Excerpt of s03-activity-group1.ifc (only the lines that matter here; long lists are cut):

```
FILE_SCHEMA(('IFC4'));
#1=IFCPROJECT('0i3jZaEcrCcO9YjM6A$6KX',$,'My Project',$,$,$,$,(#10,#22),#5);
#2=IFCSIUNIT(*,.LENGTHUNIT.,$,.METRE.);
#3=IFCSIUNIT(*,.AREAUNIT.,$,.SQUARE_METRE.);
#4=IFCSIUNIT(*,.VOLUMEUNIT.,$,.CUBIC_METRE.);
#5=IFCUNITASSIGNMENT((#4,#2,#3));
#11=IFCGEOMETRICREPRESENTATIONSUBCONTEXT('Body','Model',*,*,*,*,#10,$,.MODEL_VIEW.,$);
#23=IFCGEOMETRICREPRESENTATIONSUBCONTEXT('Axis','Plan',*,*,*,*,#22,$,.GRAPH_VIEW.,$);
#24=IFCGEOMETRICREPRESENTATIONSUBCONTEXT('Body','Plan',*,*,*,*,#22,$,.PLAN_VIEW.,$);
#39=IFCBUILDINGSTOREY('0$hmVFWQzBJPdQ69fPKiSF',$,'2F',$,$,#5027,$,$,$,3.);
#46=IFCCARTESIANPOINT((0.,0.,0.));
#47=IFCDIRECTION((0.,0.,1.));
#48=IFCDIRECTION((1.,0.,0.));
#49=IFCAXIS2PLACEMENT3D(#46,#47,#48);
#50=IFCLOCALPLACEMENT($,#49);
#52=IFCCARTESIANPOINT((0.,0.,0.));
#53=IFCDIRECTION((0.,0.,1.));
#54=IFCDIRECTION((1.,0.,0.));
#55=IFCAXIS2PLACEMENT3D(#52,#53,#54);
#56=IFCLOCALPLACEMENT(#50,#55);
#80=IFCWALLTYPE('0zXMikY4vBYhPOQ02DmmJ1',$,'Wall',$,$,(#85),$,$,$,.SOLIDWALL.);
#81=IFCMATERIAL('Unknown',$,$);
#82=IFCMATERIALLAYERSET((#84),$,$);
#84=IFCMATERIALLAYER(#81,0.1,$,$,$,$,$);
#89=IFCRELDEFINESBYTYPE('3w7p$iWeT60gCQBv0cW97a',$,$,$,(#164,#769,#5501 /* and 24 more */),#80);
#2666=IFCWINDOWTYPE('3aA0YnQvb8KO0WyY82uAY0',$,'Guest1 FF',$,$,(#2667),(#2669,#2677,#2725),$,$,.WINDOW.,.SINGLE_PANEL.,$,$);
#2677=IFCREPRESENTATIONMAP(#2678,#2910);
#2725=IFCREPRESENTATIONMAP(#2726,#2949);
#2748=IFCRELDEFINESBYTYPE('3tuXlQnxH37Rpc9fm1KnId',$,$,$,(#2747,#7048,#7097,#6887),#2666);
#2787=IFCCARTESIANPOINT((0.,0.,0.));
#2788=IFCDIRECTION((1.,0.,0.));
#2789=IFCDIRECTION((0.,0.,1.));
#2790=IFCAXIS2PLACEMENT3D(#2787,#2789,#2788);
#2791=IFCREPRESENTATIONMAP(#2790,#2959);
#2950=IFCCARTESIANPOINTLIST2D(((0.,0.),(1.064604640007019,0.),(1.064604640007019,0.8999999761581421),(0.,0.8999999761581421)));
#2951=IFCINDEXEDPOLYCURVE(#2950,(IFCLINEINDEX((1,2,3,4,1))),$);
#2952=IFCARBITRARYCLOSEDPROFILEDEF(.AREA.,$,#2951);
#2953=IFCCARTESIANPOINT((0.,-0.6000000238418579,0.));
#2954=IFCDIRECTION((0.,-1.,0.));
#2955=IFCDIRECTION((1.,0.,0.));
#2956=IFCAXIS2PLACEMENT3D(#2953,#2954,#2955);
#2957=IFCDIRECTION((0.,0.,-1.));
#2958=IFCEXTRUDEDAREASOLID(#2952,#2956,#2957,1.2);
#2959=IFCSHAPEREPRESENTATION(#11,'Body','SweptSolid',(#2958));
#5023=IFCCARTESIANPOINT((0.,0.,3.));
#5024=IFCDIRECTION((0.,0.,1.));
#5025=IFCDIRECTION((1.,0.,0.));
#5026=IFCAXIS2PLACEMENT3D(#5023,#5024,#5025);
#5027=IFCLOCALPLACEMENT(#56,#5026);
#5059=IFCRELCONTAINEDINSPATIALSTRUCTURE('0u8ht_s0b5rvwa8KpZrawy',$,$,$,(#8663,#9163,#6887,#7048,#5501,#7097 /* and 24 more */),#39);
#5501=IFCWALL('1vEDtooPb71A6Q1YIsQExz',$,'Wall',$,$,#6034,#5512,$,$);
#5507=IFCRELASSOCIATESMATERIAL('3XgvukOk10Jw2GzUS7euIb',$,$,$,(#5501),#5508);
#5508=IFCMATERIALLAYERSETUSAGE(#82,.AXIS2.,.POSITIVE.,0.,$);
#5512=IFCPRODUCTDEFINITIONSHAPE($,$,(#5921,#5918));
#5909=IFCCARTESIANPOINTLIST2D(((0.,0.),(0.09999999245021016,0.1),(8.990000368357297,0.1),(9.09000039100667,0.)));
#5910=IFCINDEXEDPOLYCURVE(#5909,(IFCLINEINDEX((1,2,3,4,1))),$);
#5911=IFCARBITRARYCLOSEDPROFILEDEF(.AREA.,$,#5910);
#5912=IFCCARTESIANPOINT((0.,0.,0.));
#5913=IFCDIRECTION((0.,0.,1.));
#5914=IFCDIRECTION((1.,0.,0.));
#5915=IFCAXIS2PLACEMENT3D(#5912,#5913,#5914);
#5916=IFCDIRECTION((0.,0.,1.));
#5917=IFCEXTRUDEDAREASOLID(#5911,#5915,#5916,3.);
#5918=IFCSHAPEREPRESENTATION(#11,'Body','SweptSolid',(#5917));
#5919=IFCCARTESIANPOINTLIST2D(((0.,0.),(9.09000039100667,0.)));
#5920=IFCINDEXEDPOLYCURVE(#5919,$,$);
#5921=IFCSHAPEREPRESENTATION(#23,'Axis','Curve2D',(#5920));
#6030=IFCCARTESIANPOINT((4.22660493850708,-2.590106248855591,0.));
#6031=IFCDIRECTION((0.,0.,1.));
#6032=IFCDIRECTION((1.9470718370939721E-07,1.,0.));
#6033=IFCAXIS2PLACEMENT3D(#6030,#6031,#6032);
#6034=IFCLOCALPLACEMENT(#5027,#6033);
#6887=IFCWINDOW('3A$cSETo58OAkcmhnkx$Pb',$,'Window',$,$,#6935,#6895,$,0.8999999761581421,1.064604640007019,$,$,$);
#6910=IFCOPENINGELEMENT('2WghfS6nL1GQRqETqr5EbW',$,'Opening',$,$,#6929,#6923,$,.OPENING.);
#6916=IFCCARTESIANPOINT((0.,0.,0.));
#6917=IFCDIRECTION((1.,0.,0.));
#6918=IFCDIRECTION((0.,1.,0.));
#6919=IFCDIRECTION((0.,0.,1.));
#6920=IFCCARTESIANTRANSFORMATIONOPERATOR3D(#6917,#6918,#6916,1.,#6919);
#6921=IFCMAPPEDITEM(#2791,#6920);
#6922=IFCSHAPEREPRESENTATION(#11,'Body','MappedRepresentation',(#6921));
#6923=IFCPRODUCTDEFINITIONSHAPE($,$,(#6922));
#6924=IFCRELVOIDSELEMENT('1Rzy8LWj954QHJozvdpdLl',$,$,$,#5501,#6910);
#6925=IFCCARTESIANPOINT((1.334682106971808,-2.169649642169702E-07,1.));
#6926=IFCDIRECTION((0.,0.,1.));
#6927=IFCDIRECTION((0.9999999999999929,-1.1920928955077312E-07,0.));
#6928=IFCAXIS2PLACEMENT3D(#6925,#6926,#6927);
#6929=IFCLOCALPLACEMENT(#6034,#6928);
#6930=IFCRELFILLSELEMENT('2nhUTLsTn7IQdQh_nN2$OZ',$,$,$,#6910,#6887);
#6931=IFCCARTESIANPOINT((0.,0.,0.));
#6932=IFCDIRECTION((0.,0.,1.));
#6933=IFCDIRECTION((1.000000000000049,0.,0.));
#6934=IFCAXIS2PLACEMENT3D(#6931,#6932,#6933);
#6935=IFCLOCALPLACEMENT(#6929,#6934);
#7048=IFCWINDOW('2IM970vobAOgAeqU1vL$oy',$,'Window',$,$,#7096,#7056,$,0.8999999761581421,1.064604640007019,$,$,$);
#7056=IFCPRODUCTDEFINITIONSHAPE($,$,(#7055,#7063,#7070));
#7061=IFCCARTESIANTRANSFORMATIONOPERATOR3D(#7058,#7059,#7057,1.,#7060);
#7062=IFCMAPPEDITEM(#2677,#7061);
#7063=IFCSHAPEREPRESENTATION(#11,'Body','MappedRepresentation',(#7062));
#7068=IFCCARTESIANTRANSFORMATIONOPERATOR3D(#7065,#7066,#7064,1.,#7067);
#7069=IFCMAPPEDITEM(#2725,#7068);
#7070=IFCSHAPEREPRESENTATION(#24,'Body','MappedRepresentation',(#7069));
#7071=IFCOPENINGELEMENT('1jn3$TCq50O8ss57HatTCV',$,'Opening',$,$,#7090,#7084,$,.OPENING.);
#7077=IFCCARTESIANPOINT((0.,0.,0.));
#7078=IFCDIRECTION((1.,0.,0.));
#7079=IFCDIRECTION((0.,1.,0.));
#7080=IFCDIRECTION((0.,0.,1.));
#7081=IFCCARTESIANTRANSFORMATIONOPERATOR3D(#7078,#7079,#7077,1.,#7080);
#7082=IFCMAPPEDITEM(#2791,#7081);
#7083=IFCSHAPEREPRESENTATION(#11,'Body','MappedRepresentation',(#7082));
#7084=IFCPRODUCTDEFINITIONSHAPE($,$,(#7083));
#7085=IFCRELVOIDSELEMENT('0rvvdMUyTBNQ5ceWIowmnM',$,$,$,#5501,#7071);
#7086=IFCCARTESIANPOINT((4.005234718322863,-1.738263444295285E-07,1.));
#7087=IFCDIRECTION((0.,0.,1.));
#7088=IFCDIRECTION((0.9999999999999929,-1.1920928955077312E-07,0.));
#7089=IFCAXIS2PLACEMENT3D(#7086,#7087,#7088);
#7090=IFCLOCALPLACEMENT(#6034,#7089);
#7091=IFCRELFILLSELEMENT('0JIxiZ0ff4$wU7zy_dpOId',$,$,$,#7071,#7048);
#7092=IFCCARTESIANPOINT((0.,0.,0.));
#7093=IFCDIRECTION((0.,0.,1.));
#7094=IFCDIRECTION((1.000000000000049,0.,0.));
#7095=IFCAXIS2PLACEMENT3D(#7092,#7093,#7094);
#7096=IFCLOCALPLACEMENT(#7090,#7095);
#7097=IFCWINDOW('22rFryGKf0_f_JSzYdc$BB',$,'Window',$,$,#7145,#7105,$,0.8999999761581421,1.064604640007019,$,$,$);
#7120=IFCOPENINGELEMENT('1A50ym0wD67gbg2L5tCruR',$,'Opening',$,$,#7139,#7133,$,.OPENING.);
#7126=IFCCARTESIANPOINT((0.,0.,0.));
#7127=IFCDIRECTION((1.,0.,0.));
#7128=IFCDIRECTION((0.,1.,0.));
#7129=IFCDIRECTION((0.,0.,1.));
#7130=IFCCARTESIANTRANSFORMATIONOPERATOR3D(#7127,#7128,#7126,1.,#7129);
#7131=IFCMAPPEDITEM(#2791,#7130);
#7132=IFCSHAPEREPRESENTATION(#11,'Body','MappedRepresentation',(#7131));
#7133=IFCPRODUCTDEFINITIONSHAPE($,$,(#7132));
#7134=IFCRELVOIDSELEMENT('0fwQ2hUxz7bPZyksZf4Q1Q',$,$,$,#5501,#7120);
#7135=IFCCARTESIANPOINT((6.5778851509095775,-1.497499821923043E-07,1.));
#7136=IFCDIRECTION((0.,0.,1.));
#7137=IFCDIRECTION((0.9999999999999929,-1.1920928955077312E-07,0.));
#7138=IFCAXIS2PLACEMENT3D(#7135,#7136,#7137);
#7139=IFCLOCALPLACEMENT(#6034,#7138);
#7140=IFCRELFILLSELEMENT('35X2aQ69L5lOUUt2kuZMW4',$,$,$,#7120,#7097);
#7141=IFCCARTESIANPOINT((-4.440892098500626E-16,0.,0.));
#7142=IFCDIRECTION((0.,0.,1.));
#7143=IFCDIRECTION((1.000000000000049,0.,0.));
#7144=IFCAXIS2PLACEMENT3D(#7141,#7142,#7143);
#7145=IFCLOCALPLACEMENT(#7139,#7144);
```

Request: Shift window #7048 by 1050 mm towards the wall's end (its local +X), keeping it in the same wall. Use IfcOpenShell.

```python
import ifcopenshell
import ifcopenshell.api.geometry
import ifcopenshell.util.placement
import ifcopenshell.util.unit

model = ifcopenshell.open("s03-activity-group1.ifc")
unit_scale = ifcopenshell.util.unit.calculate_unit_scale(model)

window = model.by_id(7048)
opening = window.FillsVoids[0].RelatingOpeningElement
wall = opening.VoidsElements[0].RelatingBuildingElement

wall_matrix = ifcopenshell.util.placement.get_local_placement(wall.ObjectPlacement)
shift = wall_matrix[:3, 0] * 1.05 / unit_scale
before = ifcopenshell.util.placement.get_local_placement(window.ObjectPlacement)[:3, 3].copy()

# The window is placed relative to its opening, so it follows when the opening moves.
matrix = ifcopenshell.util.placement.get_local_placement(opening.ObjectPlacement)
matrix[:3, 3] += shift
ifcopenshell.api.geometry.edit_object_placement(
    model, product=opening, matrix=matrix, is_si=False, should_transform_children=True
)

after = ifcopenshell.util.placement.get_local_placement(window.ObjectPlacement)[:3, 3]
print("window moved by", (after - before).round(3) + 0.0)

model.write("s03-activity-group1_v2.ifc")
```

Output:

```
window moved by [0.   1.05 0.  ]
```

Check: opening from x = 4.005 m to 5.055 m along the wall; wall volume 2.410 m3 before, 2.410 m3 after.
